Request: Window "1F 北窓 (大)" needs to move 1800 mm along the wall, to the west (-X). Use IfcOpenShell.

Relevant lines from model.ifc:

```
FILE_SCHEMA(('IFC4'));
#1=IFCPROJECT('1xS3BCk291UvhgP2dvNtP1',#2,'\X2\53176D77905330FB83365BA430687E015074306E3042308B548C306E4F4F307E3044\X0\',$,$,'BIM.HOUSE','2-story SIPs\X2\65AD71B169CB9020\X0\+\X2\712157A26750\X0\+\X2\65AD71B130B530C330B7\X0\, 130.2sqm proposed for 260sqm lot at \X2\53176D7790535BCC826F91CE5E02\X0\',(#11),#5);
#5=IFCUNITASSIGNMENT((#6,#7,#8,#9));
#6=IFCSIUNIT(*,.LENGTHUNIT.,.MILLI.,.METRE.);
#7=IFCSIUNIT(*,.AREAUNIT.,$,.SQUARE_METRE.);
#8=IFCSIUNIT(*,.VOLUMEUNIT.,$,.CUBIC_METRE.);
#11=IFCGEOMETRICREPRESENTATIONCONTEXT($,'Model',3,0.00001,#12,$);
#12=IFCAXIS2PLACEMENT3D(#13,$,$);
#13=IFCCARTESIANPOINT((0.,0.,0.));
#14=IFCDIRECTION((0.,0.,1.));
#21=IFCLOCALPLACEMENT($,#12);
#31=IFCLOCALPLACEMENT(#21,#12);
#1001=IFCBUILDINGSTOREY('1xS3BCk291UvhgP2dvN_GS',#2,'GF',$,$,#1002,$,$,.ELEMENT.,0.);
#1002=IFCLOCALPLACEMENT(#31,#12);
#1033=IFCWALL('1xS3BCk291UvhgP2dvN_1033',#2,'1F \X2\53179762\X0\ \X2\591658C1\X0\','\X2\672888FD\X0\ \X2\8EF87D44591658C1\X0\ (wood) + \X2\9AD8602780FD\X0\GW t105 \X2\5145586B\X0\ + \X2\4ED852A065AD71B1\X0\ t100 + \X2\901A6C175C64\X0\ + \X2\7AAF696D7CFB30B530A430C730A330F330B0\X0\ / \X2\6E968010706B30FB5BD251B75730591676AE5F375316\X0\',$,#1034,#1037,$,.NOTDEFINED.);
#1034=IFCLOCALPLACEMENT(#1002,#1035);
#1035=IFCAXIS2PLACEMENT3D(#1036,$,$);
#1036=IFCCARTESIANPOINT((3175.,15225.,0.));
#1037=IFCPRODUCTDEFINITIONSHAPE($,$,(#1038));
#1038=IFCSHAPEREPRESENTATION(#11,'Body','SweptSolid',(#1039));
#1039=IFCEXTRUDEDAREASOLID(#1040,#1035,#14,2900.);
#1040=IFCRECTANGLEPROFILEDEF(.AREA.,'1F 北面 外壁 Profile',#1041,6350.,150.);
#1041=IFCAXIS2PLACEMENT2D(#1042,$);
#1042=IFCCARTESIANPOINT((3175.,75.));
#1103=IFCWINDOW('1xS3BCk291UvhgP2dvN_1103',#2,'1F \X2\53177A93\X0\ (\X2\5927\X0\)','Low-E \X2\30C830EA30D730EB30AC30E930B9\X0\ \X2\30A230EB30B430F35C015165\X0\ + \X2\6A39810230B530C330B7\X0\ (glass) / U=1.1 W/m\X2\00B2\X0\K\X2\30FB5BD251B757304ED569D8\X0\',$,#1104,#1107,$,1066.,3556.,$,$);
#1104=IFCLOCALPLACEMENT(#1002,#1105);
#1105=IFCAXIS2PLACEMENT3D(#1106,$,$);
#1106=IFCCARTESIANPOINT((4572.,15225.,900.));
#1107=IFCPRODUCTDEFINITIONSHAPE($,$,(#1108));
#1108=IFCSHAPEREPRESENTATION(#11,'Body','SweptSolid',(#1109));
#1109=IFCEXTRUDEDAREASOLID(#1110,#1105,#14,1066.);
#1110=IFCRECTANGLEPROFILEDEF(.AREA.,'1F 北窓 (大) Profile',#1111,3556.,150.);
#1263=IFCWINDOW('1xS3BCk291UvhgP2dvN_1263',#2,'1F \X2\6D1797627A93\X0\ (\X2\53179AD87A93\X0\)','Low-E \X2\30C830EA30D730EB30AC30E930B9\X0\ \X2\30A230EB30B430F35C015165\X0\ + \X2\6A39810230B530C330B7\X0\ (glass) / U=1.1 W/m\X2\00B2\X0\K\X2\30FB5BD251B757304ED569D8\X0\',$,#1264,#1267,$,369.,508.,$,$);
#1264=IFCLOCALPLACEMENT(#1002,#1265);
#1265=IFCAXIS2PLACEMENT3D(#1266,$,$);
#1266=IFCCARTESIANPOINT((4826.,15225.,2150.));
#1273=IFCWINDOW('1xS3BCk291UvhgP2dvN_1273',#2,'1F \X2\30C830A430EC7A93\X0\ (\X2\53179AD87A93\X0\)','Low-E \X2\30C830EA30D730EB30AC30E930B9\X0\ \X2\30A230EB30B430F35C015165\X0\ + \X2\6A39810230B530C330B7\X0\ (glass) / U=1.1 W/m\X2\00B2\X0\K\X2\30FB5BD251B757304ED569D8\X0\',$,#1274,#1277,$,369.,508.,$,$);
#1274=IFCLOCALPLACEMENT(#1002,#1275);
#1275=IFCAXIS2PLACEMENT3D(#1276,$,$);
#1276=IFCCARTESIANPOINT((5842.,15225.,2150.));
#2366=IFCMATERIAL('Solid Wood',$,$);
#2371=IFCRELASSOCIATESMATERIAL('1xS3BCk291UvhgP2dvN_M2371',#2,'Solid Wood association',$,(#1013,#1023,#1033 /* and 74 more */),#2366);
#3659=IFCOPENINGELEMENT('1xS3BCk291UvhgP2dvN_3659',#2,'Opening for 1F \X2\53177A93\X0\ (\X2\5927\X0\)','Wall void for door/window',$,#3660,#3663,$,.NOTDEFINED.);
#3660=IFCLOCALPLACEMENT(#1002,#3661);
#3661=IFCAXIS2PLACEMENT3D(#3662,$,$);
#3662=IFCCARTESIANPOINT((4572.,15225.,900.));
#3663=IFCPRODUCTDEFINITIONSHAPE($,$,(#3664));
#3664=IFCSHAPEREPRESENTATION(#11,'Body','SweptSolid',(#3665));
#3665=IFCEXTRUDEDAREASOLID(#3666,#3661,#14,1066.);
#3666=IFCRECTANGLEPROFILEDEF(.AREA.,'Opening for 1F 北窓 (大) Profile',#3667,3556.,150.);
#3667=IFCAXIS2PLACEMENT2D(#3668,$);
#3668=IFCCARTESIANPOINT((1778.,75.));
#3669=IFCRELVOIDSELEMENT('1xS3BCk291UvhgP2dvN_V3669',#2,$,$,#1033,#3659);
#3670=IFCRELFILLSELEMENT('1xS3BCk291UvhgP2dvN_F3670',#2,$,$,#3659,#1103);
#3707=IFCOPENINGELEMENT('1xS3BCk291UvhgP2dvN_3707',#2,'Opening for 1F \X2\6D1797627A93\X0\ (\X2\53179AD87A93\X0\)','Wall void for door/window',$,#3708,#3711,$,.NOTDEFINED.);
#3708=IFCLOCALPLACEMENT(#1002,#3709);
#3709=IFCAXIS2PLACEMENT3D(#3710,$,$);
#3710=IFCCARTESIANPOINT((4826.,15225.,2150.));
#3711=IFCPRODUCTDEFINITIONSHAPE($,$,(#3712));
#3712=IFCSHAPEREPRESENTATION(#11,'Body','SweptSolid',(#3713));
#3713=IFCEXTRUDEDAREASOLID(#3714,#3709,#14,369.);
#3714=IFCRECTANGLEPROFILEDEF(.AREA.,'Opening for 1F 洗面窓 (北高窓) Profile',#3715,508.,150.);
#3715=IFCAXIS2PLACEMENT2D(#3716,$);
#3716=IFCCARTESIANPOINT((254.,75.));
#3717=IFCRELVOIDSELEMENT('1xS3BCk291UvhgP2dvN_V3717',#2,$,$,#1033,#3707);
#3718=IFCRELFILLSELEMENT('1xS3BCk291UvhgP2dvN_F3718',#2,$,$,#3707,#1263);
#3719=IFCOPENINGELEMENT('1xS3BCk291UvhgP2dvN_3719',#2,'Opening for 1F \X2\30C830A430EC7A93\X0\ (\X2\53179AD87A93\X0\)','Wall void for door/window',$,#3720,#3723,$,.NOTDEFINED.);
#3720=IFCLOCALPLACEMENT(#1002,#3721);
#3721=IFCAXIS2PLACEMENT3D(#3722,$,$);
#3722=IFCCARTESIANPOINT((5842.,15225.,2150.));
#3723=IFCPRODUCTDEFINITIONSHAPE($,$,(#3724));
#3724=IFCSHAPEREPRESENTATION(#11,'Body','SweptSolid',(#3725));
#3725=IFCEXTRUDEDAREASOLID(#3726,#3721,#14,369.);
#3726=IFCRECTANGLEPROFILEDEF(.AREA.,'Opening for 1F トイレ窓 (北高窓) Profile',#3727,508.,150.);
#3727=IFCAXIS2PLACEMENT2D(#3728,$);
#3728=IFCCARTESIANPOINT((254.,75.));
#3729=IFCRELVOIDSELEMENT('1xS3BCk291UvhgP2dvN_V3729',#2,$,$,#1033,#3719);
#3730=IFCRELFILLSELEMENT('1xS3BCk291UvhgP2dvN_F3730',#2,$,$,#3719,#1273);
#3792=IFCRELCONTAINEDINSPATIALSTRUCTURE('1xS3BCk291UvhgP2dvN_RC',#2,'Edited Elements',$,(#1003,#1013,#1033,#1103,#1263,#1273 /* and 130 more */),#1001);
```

```python
import ifcopenshell
import ifcopenshell.api.geometry
import ifcopenshell.util.placement
import ifcopenshell.util.unit

model = ifcopenshell.open("model.ifc")
unit_scale = ifcopenshell.util.unit.calculate_unit_scale(model)

window = model.by_id(1103)
opening = window.FillsVoids[0].RelatingOpeningElement
wall = opening.VoidsElements[0].RelatingBuildingElement

wall_matrix = ifcopenshell.util.placement.get_local_placement(wall.ObjectPlacement)
shift = wall_matrix[:3, 0] * -1.8 / unit_scale
before = ifcopenshell.util.placement.get_local_placement(window.ObjectPlacement)[:3, 3].copy()

# The window is not placed relative to its opening, so move both.
for product in (opening, window):
    matrix = ifcopenshell.util.placement.get_local_placement(product.ObjectPlacement)
    matrix[:3, 3] += shift
    ifcopenshell.api.geometry.edit_object_placement(model, product=product, matrix=matrix, is_si=False)

after = ifcopenshell.util.placement.get_local_placement(window.ObjectPlacement)[:3, 3]
print("window moved by", (after - before).round(3) + 0.0)

model.write("model-out.ifc")
```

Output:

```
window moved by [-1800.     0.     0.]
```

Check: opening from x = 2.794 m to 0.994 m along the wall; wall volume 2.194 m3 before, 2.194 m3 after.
